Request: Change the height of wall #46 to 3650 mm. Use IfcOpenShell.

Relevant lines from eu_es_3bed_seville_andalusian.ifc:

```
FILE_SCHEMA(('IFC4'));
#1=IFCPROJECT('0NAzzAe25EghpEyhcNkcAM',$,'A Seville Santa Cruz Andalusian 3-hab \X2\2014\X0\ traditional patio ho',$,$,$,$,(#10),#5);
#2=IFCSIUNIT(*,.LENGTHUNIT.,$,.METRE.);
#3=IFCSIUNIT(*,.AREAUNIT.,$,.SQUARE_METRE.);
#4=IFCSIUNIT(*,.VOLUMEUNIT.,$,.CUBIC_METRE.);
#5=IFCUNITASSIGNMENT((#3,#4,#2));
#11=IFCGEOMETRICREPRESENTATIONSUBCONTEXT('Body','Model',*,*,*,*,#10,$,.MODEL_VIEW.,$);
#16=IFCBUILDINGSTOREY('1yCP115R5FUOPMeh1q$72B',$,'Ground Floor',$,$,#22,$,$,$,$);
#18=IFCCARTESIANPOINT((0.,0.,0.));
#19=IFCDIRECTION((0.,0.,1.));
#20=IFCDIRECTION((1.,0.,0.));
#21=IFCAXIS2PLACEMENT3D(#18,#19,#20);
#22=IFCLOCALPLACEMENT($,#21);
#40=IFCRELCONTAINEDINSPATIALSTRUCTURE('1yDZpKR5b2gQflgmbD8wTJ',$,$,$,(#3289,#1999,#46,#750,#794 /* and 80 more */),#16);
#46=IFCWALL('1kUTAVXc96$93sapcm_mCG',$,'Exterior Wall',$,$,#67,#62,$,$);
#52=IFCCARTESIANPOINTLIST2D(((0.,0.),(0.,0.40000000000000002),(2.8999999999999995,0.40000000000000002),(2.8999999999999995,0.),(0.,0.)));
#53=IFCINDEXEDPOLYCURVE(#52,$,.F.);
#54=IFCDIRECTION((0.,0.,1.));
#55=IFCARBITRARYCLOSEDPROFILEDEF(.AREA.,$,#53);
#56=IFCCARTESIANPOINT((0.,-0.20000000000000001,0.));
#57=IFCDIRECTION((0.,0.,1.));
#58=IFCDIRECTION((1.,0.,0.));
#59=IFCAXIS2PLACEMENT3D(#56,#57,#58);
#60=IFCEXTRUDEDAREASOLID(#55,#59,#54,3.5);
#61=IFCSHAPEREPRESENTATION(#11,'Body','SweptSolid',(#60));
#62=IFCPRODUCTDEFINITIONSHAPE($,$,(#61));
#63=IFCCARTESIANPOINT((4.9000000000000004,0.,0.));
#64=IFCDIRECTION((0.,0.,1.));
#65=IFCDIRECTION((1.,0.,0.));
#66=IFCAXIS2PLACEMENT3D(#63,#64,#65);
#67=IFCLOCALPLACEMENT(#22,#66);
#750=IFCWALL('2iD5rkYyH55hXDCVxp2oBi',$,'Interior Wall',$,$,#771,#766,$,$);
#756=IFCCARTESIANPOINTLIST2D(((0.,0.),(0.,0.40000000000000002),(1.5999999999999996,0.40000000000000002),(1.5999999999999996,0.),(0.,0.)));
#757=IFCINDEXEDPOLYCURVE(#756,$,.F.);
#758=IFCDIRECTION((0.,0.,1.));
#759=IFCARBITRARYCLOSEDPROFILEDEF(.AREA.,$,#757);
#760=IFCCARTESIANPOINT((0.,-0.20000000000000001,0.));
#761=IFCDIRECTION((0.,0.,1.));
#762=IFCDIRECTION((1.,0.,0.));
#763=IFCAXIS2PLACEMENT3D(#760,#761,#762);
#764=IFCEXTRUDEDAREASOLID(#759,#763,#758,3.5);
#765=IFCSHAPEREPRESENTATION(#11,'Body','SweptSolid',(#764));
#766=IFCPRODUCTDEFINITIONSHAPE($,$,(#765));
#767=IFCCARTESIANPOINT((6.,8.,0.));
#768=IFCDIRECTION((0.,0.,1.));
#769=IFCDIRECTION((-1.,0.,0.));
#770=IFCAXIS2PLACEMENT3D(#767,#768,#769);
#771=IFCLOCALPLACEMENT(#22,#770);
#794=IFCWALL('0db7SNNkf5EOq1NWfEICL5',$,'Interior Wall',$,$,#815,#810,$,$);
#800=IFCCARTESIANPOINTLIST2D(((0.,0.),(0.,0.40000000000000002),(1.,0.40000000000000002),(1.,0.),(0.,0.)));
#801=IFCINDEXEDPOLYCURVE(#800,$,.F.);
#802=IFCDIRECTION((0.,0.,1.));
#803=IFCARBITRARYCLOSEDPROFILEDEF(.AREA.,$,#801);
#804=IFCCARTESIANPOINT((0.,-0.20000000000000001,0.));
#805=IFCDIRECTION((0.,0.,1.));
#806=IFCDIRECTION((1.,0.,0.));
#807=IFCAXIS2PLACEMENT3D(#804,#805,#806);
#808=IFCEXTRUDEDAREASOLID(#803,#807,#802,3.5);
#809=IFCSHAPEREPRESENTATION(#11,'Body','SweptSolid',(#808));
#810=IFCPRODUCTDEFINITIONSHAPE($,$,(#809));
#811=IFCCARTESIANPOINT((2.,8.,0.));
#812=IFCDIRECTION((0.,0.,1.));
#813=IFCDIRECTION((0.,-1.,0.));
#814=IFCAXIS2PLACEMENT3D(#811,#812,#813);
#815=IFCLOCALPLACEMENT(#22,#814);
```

```python
import ifcopenshell
import ifcopenshell.geom
import ifcopenshell.util.representation
import ifcopenshell.util.shape

model = ifcopenshell.open("eu_es_3bed_seville_andalusian.ifc")
settings = ifcopenshell.geom.settings()


def volume(element):
    """Net volume in cubic metres, openings subtracted."""
    shape = ifcopenshell.geom.create_shape(settings, element)
    return ifcopenshell.util.shape.get_volume(shape.geometry)


wall = model.by_guid("1kUTAVXc96$93sapcm_mCG")
before = volume(wall)

body = ifcopenshell.util.representation.get_representation(wall, "Model", "Body")
solid = body.Items[0]
old_height = solid.Depth
solid.Depth = 3.65
after = volume(wall)

print(f"height {old_height:g} -> {solid.Depth:g}, volume {before:.3f} -> {after:.3f} m3")

model.write("eu_es_3bed_seville_andalusian_edited.ifc")
```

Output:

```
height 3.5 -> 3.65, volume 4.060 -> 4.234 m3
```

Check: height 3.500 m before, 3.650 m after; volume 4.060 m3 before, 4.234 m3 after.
